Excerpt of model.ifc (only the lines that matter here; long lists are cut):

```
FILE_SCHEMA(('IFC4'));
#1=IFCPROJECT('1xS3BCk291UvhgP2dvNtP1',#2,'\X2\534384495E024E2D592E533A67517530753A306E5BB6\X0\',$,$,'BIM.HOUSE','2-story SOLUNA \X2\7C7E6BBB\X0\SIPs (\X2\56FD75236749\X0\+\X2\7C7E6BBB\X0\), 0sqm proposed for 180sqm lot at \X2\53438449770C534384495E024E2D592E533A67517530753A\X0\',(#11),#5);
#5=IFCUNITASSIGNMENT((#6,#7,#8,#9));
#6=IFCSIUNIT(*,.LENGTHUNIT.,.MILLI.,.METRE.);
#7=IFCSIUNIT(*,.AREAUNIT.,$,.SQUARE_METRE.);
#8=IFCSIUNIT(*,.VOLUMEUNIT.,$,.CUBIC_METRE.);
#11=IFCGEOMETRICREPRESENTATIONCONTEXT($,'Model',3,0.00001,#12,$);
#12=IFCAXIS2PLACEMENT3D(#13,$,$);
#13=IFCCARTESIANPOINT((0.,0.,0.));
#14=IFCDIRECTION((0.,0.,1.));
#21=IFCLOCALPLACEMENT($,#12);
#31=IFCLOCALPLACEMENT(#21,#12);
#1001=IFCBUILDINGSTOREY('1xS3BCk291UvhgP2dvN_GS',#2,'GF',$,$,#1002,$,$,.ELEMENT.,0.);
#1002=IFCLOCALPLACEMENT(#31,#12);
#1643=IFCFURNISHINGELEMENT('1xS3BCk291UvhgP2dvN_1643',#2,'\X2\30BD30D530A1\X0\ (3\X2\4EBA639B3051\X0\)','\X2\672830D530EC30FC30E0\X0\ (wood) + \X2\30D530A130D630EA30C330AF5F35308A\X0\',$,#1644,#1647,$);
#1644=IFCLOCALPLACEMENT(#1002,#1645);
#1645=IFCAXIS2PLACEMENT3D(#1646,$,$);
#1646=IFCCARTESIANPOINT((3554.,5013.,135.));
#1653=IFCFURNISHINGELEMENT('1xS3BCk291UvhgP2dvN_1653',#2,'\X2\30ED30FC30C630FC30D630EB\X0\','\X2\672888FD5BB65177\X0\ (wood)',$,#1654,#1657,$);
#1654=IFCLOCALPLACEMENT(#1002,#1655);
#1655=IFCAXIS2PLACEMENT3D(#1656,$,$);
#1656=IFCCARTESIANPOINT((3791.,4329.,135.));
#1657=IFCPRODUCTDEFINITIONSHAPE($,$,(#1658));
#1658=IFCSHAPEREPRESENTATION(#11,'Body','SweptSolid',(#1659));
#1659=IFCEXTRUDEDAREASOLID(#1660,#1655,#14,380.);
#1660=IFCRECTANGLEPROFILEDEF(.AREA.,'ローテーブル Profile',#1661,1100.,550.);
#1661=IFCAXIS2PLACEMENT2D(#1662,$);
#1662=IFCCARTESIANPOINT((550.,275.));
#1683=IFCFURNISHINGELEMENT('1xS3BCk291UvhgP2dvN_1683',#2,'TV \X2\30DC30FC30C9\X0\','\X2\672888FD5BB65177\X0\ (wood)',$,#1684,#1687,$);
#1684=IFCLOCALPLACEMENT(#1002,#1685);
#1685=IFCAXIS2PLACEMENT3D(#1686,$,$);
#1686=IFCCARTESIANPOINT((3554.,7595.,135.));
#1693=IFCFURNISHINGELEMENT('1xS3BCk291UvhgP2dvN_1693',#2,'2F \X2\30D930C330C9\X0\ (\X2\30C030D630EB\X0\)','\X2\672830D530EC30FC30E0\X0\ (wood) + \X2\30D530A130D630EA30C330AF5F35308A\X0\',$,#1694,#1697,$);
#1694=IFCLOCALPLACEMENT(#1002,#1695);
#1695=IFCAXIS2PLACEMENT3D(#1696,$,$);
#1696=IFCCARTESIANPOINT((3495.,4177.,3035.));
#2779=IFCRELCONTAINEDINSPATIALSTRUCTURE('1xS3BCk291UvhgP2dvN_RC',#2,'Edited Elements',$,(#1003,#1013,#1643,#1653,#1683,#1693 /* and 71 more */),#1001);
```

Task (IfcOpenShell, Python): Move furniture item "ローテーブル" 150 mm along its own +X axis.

```python
import ifcopenshell
import ifcopenshell.api.geometry
import ifcopenshell.util.placement
import ifcopenshell.util.unit

model = ifcopenshell.open("model.ifc")
unit_scale = ifcopenshell.util.unit.calculate_unit_scale(model)

item = model.by_guid("1xS3BCk291UvhgP2dvN_1653")
matrix = ifcopenshell.util.placement.get_local_placement(item.ObjectPlacement)
matrix[:3, 3] += matrix[:3, 0] * 0.15 / unit_scale
ifcopenshell.api.geometry.edit_object_placement(model, product=item, matrix=matrix, is_si=False)

print(ifcopenshell.util.placement.get_local_placement(item.ObjectPlacement).round(3) + 0.0)

model.write("model_updated.ifc")
```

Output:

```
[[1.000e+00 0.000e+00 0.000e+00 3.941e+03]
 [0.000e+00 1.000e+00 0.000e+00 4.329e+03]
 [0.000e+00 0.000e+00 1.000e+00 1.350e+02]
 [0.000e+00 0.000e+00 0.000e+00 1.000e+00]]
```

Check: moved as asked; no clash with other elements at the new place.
